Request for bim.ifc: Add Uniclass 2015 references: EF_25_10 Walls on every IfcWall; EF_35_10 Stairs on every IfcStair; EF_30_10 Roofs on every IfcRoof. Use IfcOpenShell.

First a look at what the model holds.

```python
import ifcopenshell

model = ifcopenshell.open("bim.ifc")
print(model.schema)
print("classifications:", [c.Name for c in model.by_type("IfcClassification")])
for ifc_class in ("IfcDoor", "IfcRoof", "IfcStair", "IfcWall", "IfcWindow"):
    print(ifc_class, len(model.by_type(ifc_class)))
```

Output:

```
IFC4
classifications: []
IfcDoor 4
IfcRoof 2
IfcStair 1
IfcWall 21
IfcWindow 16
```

```python
import ifcopenshell
import ifcopenshell.api.classification

model = ifcopenshell.open("bim.ifc")

system = ifcopenshell.api.classification.add_classification(model, classification="Uniclass 2015")

codes = {
    "IfcWall": ("EF_25_10", "Walls"),
    "IfcStair": ("EF_35_10", "Stairs"),
    "IfcRoof": ("EF_30_10", "Roofs"),
}
for ifc_class, (code, name) in codes.items():
    products = model.by_type(ifc_class)
    ifcopenshell.api.classification.add_reference(
        model, products=products, classification=system, identification=code, name=name
    )
    print(code, len(products))

model.write("bim_updated.ifc")
```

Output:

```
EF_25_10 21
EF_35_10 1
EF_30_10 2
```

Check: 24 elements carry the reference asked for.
